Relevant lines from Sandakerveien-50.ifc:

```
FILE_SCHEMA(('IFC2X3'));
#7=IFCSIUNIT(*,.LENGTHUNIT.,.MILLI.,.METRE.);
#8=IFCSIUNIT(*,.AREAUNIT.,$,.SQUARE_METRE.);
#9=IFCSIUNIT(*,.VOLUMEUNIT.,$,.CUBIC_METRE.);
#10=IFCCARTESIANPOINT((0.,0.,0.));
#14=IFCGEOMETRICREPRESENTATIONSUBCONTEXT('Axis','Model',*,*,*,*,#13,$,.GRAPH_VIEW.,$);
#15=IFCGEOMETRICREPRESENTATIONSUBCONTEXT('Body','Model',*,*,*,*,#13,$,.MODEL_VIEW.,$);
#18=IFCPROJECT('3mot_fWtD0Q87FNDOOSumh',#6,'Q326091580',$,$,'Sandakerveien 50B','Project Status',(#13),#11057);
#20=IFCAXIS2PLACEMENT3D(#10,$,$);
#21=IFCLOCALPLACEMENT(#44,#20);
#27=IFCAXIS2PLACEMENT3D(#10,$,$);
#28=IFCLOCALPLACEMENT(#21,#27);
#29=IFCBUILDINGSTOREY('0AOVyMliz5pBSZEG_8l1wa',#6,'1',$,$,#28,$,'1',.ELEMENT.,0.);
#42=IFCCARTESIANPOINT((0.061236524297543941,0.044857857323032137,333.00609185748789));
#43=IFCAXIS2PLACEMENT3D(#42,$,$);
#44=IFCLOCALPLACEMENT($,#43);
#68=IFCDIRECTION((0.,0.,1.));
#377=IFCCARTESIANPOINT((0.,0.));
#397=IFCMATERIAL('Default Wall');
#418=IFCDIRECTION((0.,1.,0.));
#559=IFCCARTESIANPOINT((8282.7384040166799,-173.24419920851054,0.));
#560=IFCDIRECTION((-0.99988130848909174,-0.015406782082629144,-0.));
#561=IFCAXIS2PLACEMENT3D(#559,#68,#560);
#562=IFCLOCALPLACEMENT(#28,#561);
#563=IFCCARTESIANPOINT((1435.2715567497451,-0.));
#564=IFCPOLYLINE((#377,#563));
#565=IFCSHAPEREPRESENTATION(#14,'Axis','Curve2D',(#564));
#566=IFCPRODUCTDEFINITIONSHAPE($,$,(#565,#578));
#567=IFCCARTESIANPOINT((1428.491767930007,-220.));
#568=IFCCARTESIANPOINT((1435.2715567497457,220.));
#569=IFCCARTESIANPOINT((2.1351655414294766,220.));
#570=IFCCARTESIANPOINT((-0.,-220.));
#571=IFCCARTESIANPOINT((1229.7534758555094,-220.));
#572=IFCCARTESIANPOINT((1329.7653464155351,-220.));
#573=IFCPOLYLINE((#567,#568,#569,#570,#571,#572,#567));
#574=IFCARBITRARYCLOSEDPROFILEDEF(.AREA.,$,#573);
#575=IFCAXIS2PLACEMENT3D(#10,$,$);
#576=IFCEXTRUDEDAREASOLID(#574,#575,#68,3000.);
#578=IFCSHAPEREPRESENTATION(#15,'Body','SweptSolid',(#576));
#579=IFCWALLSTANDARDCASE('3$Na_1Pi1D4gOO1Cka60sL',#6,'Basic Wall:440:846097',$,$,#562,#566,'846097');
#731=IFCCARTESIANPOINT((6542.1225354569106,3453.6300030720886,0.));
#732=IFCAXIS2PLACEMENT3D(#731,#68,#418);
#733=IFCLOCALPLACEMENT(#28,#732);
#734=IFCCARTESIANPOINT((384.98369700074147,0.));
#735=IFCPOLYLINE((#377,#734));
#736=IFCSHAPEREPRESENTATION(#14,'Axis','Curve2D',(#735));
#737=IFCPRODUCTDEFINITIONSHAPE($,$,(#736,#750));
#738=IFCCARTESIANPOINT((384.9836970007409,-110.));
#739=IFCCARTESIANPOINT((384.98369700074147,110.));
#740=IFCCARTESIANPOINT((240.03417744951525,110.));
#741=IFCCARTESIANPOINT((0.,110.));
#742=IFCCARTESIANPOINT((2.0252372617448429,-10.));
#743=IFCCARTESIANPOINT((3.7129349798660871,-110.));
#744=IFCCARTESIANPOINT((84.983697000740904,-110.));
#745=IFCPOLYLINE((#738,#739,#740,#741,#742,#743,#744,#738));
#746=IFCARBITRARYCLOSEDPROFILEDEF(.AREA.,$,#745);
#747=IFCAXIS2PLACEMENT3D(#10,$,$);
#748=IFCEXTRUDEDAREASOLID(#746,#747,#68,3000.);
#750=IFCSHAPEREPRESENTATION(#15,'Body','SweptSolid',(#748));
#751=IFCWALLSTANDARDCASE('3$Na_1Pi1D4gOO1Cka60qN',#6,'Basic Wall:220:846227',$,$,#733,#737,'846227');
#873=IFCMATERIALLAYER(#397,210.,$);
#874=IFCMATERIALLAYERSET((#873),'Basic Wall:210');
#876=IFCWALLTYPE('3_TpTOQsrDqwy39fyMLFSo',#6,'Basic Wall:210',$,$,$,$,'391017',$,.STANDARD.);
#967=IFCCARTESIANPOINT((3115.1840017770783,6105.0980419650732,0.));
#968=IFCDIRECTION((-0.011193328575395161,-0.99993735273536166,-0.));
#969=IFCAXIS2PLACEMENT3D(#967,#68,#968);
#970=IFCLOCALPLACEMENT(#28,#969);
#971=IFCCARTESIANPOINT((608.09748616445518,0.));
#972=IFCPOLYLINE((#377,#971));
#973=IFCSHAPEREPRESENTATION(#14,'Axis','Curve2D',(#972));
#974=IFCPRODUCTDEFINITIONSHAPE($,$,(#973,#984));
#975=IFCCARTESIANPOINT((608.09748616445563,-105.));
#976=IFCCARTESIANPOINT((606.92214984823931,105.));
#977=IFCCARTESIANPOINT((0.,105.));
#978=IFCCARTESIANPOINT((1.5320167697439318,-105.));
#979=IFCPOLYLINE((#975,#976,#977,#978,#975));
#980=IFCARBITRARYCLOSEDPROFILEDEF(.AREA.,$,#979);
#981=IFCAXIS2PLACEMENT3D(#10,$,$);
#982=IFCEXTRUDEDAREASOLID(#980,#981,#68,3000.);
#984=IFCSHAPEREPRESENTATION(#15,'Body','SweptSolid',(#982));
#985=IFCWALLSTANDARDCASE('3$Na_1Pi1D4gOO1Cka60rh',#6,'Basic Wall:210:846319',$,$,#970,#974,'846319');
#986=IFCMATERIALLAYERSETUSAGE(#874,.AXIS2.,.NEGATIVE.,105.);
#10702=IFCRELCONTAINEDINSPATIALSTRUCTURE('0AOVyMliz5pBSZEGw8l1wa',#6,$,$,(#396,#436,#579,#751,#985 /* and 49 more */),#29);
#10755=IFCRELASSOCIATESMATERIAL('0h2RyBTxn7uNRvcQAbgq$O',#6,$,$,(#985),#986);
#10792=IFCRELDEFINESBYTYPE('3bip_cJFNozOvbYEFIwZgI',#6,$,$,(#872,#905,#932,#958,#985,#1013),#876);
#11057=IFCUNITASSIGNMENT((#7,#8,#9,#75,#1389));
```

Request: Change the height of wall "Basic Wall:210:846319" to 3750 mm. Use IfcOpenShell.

```python
import ifcopenshell
import ifcopenshell.geom
import ifcopenshell.util.representation
import ifcopenshell.util.shape
import ifcopenshell.util.unit

model = ifcopenshell.open("Sandakerveien-50.ifc")
unit_scale = ifcopenshell.util.unit.calculate_unit_scale(model)
settings = ifcopenshell.geom.settings()


def volume(element):
    """Net volume in cubic metres, openings subtracted."""
    shape = ifcopenshell.geom.create_shape(settings, element)
    return ifcopenshell.util.shape.get_volume(shape.geometry)


wall = model.by_guid("3$Na_1Pi1D4gOO1Cka60rh")
before = volume(wall)

body = ifcopenshell.util.representation.get_representation(wall, "Model", "Body")
solid = body.Items[0]
old_height = solid.Depth
solid.Depth = 3.75 / unit_scale
after = volume(wall)

print(f"height {old_height:g} -> {solid.Depth:g}, volume {before:.3f} -> {after:.3f} m3")

model.write("Sandakerveien-50_v2.ifc")
```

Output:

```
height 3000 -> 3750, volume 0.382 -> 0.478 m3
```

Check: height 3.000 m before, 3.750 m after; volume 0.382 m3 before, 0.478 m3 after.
